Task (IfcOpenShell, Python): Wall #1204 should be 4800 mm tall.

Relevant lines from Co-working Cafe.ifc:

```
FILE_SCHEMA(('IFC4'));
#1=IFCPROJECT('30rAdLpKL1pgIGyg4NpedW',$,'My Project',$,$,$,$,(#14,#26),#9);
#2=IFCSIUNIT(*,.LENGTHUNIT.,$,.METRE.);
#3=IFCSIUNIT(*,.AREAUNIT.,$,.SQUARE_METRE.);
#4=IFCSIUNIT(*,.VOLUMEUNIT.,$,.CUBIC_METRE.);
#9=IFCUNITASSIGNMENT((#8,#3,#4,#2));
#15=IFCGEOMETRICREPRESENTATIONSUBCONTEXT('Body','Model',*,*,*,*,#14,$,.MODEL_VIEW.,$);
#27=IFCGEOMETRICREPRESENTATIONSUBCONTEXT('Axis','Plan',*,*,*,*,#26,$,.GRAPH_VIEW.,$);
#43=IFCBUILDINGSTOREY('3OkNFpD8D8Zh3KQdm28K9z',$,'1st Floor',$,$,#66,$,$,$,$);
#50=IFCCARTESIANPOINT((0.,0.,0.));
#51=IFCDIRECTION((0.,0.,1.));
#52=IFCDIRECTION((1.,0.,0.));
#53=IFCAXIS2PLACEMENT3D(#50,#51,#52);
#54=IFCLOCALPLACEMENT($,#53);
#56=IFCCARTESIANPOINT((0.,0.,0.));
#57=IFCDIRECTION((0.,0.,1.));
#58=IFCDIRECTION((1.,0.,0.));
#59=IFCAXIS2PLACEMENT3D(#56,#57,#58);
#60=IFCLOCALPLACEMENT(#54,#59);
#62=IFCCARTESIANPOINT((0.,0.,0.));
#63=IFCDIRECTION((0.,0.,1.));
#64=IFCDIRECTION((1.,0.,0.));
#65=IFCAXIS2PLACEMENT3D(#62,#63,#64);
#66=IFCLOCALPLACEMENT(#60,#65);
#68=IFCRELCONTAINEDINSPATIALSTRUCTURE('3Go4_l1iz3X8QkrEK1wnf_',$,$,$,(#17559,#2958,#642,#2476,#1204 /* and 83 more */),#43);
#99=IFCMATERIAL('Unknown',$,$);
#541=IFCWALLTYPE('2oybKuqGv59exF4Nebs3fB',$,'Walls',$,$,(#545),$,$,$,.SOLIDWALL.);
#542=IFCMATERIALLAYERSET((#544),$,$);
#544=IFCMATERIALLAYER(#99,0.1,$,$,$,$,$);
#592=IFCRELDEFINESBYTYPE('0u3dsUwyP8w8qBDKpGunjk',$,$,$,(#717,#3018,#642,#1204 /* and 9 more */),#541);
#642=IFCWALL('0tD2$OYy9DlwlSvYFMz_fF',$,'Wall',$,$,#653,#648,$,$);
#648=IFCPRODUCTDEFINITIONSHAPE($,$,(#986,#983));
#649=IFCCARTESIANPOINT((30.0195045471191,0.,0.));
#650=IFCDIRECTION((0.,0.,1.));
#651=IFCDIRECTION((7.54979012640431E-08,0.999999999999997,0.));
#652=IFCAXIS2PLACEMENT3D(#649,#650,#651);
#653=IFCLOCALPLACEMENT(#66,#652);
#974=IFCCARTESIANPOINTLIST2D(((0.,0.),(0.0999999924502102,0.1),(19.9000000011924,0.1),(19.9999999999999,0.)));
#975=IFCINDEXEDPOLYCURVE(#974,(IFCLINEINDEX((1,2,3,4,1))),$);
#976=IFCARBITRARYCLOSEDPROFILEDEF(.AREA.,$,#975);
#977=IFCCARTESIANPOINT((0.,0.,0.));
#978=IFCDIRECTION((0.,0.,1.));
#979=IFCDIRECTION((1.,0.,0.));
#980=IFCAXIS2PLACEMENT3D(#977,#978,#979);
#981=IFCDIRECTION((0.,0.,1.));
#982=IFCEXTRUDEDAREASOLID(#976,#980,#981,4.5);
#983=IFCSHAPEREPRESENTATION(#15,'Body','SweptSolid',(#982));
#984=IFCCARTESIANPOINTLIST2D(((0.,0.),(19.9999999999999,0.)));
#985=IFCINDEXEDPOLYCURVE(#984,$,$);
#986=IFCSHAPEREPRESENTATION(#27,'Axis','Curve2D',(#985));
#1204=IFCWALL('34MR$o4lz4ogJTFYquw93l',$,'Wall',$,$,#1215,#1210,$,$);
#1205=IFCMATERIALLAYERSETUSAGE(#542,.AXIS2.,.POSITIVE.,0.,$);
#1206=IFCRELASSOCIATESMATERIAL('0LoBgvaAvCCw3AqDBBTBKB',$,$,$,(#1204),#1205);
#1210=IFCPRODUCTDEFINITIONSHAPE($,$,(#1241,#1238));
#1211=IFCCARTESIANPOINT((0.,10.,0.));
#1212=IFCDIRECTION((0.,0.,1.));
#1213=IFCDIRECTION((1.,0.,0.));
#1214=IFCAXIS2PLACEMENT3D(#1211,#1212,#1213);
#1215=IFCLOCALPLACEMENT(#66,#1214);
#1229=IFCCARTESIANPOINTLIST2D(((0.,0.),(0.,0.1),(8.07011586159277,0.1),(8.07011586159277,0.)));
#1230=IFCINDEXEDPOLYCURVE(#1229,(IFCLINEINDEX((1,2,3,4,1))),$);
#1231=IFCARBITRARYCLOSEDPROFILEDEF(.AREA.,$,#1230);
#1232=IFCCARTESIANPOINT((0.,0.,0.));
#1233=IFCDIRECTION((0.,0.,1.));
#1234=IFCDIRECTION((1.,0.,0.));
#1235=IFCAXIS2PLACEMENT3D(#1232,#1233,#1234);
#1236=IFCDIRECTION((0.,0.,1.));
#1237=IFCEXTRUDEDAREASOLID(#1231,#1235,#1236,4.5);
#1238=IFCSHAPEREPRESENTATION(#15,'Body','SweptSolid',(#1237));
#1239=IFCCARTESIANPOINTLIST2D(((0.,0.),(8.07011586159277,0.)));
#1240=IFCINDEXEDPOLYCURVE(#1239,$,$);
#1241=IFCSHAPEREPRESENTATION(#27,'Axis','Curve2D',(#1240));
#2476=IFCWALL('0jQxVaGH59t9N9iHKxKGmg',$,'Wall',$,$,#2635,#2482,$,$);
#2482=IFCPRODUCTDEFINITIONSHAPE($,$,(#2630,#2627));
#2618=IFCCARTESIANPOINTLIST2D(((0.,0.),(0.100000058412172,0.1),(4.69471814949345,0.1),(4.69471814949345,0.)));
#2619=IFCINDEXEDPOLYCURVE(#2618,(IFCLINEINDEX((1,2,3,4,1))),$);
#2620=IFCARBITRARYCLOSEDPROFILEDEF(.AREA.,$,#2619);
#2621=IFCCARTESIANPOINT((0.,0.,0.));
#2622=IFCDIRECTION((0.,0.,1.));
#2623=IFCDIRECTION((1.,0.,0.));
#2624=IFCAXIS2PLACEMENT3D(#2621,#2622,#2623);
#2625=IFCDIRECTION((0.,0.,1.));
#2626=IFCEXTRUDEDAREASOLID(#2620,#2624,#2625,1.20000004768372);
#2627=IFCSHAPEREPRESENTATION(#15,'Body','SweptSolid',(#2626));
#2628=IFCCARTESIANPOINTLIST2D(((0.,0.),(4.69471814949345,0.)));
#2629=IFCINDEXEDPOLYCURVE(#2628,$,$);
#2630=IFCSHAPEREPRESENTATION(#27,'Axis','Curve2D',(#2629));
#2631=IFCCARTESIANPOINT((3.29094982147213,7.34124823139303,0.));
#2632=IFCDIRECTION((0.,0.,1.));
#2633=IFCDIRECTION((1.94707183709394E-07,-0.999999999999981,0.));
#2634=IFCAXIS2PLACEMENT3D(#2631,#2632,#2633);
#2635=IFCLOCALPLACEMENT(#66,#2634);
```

```python
import ifcopenshell
import ifcopenshell.geom
import ifcopenshell.util.representation
import ifcopenshell.util.shape

model = ifcopenshell.open("Co-working Cafe.ifc")
settings = ifcopenshell.geom.settings()


def volume(element):
    """Net volume in cubic metres, openings subtracted."""
    shape = ifcopenshell.geom.create_shape(settings, element)
    return ifcopenshell.util.shape.get_volume(shape.geometry)


wall = model.by_guid("34MR$o4lz4ogJTFYquw93l")
before = volume(wall)

body = ifcopenshell.util.representation.get_representation(wall, "Model", "Body")
solid = body.Items[0]
old_height = solid.Depth
solid.Depth = 4.8
after = volume(wall)

print(f"height {old_height:g} -> {solid.Depth:g}, volume {before:.3f} -> {after:.3f} m3")

model.write("Co-working Cafe_rev.ifc")
```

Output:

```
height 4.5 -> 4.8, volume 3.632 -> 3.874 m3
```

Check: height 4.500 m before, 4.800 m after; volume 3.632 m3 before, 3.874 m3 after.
